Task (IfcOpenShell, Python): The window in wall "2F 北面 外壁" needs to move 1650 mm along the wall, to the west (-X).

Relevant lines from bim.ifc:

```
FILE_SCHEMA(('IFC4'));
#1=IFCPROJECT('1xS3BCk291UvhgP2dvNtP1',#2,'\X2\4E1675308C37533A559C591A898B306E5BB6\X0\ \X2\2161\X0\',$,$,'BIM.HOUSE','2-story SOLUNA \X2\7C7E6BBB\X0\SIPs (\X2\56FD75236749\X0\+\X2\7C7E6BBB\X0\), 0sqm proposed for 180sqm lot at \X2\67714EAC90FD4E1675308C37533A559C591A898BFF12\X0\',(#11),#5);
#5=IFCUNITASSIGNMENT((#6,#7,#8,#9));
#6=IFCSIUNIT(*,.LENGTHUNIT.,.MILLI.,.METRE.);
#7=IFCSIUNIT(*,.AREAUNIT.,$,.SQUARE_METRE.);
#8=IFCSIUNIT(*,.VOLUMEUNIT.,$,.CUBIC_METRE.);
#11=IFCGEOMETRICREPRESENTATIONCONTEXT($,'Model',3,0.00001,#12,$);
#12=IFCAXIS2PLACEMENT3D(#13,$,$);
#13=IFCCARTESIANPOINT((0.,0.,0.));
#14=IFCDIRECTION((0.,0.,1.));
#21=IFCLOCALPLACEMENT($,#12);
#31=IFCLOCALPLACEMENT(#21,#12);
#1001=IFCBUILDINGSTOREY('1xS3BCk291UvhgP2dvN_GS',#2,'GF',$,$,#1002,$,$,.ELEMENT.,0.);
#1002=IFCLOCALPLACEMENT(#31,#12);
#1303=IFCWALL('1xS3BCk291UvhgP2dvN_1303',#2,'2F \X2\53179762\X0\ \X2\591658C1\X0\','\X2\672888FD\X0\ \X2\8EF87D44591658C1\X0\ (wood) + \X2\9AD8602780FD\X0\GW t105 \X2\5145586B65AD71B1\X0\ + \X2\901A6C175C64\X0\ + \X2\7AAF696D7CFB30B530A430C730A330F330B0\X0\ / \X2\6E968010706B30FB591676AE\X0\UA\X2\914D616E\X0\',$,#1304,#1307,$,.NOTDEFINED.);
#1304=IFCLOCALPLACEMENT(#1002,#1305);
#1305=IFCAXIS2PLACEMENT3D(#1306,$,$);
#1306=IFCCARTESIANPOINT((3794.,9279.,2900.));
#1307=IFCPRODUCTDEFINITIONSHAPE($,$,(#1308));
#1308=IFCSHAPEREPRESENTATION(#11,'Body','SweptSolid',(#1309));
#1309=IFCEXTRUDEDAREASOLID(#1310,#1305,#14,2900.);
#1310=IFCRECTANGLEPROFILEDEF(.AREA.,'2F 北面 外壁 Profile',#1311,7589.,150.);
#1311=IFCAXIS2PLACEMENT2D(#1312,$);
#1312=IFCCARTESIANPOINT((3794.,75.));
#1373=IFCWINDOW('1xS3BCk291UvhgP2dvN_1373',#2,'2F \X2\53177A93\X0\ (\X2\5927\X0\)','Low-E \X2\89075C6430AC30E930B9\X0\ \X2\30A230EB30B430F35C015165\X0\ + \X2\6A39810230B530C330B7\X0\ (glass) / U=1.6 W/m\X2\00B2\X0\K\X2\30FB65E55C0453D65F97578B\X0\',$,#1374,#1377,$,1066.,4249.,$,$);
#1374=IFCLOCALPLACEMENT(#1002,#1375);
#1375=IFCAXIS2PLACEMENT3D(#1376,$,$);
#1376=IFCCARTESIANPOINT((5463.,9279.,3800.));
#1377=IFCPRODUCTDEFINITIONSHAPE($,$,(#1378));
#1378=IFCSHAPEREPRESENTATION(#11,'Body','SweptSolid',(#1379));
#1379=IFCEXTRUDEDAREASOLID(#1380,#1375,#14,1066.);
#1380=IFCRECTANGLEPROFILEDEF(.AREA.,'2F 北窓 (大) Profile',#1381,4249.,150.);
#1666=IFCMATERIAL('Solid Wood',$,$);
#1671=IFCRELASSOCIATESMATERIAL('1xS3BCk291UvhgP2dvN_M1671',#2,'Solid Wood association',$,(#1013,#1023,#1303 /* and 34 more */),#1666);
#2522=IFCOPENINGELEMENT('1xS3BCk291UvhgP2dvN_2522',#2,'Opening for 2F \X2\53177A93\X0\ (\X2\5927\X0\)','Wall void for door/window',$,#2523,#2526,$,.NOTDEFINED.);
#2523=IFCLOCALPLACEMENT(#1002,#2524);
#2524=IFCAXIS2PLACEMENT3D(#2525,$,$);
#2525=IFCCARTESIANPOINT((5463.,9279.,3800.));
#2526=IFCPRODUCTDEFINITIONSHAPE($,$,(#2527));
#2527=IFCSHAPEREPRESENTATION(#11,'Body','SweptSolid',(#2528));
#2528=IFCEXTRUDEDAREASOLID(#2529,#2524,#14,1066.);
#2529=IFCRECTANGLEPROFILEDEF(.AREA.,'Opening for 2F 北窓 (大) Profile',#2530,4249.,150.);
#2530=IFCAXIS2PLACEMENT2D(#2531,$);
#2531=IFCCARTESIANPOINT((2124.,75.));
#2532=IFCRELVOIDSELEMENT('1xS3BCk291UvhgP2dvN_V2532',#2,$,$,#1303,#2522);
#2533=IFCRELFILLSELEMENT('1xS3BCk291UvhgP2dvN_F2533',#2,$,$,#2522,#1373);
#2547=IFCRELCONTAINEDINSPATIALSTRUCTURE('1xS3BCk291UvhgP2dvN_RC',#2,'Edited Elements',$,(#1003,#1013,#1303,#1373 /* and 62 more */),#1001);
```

```python
import ifcopenshell
import ifcopenshell.api.geometry
import ifcopenshell.util.placement

model = ifcopenshell.open("bim.ifc")

window = model.by_guid("1xS3BCk291UvhgP2dvN_1373")
opening = window.FillsVoids[0].RelatingOpeningElement
wall = opening.VoidsElements[0].RelatingBuildingElement

wall_matrix = ifcopenshell.util.placement.get_local_placement(wall.ObjectPlacement)
shift = wall_matrix[:3, 0] * -1650.0
before = ifcopenshell.util.placement.get_local_placement(window.ObjectPlacement)[:3, 3].copy()

# The window is not placed relative to its opening, so move both.
for product in (opening, window):
    matrix = ifcopenshell.util.placement.get_local_placement(product.ObjectPlacement)
    matrix[:3, 3] += shift
    ifcopenshell.api.geometry.edit_object_placement(model, product=product, matrix=matrix, is_si=False)

after = ifcopenshell.util.placement.get_local_placement(window.ObjectPlacement)[:3, 3]
print("window moved by", (after - before).round(3) + 0.0)

model.write("bim_updated.ifc")
```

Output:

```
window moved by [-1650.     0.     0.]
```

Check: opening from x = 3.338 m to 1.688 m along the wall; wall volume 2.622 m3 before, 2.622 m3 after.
